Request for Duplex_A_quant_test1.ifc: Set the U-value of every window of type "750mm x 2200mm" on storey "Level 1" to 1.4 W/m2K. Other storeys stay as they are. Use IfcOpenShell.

First a look at what the model holds.

```python
import ifcopenshell
import ifcopenshell.util.element

model = ifcopenshell.open("Duplex_A_quant_test1.ifc")
print(model.schema)
storey = next(s for s in model.by_type("IfcBuildingStorey") if s.Name == "Level 1")
windows = [e for e in ifcopenshell.util.element.get_decomposition(storey) if e.is_a("IfcWindow")]
seen = {}
for e in windows:
    element_type = ifcopenshell.util.element.get_type(e)
    key = (element_type.Name if element_type != e and element_type else None, ifcopenshell.util.element.get_pset(e, "Pset_WindowCommon", "ThermalTransmittance"))
    seen[key] = seen.get(key, 0) + 1
for (name, value), count in sorted(seen.items(), key=str):
    print(count, "x", name, "|", value)
```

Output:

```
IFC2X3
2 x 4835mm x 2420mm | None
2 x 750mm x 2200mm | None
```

```python
import ifcopenshell
import ifcopenshell.api.pset
import ifcopenshell.util.element

model = ifcopenshell.open("Duplex_A_quant_test1.ifc")

storey = next(s for s in model.by_type("IfcBuildingStorey") if s.Name == "Level 1")
windows = [e for e in ifcopenshell.util.element.get_decomposition(storey) if e.is_a("IfcWindow")]

count = 0
for e in windows:
    element_type = ifcopenshell.util.element.get_type(e)
    if element_type in (None, e) or element_type.Name != "750mm x 2200mm":
        continue
    # add_pset returns the element's existing set when there is one.
    pset = ifcopenshell.api.pset.add_pset(model, product=e, name="Pset_WindowCommon")
    ifcopenshell.api.pset.edit_pset(model, pset=pset, properties={"ThermalTransmittance": 1.4})
    count += 1

print(count, "windows updated")

model.write("Duplex_A_quant_test1_rev.ifc")
```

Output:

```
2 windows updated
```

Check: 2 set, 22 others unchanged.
